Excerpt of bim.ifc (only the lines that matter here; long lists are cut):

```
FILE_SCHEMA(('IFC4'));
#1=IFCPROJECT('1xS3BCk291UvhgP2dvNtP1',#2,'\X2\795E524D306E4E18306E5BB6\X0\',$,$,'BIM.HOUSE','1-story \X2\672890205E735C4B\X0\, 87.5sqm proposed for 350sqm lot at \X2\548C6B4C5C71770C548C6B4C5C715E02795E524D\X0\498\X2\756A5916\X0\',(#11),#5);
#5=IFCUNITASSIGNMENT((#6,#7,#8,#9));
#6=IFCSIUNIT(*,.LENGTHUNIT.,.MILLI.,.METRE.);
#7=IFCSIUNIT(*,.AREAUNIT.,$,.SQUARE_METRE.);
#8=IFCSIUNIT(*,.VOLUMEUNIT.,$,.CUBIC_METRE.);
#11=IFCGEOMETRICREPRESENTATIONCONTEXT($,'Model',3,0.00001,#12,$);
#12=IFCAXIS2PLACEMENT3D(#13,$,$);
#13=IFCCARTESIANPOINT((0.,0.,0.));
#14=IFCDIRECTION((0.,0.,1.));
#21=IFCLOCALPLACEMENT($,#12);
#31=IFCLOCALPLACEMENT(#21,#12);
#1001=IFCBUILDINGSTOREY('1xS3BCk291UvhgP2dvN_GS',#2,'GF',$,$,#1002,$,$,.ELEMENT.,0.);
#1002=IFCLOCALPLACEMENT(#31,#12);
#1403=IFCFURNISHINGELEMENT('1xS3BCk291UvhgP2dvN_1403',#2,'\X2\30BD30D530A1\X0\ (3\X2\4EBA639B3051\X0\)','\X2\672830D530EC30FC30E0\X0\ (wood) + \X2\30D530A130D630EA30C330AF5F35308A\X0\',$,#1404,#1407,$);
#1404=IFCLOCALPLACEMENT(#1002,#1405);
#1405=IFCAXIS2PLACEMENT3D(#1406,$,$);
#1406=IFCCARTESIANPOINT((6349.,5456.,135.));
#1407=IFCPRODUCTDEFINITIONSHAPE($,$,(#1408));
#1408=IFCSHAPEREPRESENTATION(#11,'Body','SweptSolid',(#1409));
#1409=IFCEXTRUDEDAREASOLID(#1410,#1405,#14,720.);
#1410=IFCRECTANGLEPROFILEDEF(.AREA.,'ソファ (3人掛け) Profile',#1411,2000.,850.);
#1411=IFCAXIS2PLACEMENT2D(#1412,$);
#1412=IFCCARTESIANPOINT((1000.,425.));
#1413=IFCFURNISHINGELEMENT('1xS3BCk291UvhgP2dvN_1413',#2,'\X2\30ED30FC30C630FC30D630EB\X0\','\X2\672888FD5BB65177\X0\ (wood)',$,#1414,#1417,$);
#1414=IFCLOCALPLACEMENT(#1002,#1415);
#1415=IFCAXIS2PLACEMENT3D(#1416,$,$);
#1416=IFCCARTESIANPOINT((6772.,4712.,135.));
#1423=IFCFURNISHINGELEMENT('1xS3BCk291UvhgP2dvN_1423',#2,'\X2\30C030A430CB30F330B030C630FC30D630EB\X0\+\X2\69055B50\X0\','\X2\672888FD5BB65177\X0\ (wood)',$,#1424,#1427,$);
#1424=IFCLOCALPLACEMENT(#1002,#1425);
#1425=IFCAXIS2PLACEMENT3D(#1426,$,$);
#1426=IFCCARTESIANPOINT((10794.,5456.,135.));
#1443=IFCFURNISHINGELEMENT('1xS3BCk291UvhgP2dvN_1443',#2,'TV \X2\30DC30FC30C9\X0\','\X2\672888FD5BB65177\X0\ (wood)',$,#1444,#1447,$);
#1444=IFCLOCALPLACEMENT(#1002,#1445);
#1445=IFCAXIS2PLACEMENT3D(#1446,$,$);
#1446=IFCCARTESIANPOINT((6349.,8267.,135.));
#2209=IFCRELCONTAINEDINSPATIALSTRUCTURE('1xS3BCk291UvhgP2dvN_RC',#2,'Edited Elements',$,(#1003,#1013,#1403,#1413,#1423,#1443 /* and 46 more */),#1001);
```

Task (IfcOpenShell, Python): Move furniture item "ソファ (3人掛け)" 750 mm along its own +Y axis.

```python
import ifcopenshell
import ifcopenshell.api.geometry
import ifcopenshell.util.placement
import ifcopenshell.util.unit

model = ifcopenshell.open("bim.ifc")
unit_scale = ifcopenshell.util.unit.calculate_unit_scale(model)

item = model.by_guid("1xS3BCk291UvhgP2dvN_1403")
matrix = ifcopenshell.util.placement.get_local_placement(item.ObjectPlacement)
matrix[:3, 3] += matrix[:3, 1] * 0.75 / unit_scale
ifcopenshell.api.geometry.edit_object_placement(model, product=item, matrix=matrix, is_si=False)

print(ifcopenshell.util.placement.get_local_placement(item.ObjectPlacement).round(3) + 0.0)

model.write("bim_updated.ifc")
```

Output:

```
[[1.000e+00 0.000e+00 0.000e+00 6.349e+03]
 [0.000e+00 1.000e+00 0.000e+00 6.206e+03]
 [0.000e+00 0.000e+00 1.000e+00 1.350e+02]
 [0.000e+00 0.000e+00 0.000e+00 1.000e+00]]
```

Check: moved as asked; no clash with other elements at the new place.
